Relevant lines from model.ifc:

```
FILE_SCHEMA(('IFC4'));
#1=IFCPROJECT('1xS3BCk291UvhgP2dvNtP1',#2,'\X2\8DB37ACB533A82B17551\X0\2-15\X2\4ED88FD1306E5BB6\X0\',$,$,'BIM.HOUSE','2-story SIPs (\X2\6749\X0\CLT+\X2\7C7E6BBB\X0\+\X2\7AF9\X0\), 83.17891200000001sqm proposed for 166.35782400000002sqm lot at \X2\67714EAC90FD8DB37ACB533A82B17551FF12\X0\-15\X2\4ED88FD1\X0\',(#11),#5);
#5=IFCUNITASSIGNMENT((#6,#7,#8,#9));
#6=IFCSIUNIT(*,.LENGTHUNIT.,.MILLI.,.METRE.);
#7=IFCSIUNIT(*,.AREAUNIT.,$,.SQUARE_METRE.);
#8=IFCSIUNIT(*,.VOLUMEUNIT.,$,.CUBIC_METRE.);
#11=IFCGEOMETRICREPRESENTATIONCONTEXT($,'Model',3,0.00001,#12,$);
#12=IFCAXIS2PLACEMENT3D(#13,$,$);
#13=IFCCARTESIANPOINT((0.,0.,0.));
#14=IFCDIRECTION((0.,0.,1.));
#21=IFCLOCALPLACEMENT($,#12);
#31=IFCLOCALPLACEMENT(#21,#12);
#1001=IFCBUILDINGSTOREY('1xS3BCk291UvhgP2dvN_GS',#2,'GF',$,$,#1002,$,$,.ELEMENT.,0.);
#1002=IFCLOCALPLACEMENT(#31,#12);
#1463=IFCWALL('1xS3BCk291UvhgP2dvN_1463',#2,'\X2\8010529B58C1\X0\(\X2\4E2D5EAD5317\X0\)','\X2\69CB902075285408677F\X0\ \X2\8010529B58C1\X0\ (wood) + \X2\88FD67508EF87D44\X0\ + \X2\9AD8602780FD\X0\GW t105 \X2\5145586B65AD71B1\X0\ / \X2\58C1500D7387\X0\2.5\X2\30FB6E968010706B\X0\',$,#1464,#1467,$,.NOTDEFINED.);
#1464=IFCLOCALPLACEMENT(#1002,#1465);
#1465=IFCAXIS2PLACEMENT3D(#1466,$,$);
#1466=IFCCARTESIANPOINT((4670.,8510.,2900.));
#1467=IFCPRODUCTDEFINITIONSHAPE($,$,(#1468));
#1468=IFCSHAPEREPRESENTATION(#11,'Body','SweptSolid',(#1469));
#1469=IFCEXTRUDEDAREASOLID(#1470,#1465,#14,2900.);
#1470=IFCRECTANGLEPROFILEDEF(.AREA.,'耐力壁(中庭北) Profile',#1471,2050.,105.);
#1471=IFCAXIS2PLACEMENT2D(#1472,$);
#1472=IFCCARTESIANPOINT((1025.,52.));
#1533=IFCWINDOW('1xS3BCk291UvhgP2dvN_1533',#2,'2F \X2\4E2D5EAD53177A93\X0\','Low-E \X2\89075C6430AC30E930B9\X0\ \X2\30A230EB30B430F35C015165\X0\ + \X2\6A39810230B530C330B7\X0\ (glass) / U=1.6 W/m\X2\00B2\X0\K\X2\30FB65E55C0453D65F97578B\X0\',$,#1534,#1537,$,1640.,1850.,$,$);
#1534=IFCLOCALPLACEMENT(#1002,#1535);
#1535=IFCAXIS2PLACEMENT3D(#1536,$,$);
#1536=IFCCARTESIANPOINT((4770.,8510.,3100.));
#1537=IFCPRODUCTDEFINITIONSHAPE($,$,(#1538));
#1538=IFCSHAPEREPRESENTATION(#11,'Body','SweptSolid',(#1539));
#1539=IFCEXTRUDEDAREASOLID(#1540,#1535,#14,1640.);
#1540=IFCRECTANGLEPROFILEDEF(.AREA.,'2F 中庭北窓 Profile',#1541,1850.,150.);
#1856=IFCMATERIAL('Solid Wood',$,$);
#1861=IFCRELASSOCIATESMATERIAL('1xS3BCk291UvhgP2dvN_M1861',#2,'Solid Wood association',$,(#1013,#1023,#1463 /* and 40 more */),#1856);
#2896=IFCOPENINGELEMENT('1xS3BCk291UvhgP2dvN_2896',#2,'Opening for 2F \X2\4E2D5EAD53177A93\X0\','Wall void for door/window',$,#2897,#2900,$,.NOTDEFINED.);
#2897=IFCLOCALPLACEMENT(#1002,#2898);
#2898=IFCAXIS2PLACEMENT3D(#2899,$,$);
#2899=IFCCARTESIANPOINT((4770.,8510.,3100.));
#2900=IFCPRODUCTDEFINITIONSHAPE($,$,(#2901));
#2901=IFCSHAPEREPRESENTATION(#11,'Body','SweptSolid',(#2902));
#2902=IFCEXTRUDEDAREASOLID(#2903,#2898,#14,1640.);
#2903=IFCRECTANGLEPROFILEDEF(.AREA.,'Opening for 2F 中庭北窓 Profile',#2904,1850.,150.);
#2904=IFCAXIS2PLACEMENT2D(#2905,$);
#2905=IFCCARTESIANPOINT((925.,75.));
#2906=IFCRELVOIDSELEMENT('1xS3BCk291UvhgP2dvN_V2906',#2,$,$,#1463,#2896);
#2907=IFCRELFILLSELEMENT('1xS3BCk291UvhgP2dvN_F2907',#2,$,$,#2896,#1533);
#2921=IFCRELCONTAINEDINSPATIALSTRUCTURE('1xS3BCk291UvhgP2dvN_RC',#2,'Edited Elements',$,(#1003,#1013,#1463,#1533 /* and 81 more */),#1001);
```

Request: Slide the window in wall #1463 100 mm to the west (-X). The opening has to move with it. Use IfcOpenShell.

```python
import ifcopenshell
import ifcopenshell.api.geometry
import ifcopenshell.util.placement
import ifcopenshell.util.unit

model = ifcopenshell.open("model.ifc")
unit_scale = ifcopenshell.util.unit.calculate_unit_scale(model)

window = model.by_guid("1xS3BCk291UvhgP2dvN_1533")
opening = window.FillsVoids[0].RelatingOpeningElement
wall = opening.VoidsElements[0].RelatingBuildingElement

wall_matrix = ifcopenshell.util.placement.get_local_placement(wall.ObjectPlacement)
shift = wall_matrix[:3, 0] * -0.1 / unit_scale
before = ifcopenshell.util.placement.get_local_placement(window.ObjectPlacement)[:3, 3].copy()

# The window is not placed relative to its opening, so move both.
for product in (opening, window):
    matrix = ifcopenshell.util.placement.get_local_placement(product.ObjectPlacement)
    matrix[:3, 3] += shift
    ifcopenshell.api.geometry.edit_object_placement(model, product=product, matrix=matrix, is_si=False)

after = ifcopenshell.util.placement.get_local_placement(window.ObjectPlacement)[:3, 3]
print("window moved by", (after - before).round(3) + 0.0)

model.write("model_v2.ifc")
```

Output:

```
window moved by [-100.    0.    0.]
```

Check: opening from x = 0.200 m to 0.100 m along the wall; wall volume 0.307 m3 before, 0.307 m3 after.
